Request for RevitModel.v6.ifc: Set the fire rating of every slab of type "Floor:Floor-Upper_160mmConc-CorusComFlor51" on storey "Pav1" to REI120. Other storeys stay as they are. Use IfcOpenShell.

First a look at what the model holds.

```python
import ifcopenshell
import ifcopenshell.util.element

model = ifcopenshell.open("RevitModel.v6.ifc")
print(model.schema)
storey = next(s for s in model.by_type("IfcBuildingStorey") if s.Name == "Pav1")
slabs = [e for e in ifcopenshell.util.element.get_decomposition(storey) if e.is_a("IfcSlab")]
seen = {}
for e in slabs:
    element_type = ifcopenshell.util.element.get_type(e)
    key = (element_type.Name if element_type != e and element_type else None, ifcopenshell.util.element.get_pset(e, "Pset_SlabCommon", "FireRating"))
    seen[key] = seen.get(key, 0) + 1
for (name, value), count in sorted(seen.items(), key=str):
    print(count, "x", name, "|", value)
```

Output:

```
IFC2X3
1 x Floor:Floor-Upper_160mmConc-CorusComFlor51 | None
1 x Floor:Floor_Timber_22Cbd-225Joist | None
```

```python
import ifcopenshell
import ifcopenshell.api.pset
import ifcopenshell.util.element

model = ifcopenshell.open("RevitModel.v6.ifc")

storey = next(s for s in model.by_type("IfcBuildingStorey") if s.Name == "Pav1")
slabs = [e for e in ifcopenshell.util.element.get_decomposition(storey) if e.is_a("IfcSlab")]

count = 0
for e in slabs:
    element_type = ifcopenshell.util.element.get_type(e)
    if element_type in (None, e) or element_type.Name != "Floor:Floor-Upper_160mmConc-CorusComFlor51":
        continue
    # add_pset returns the element's existing set when there is one.
    pset = ifcopenshell.api.pset.add_pset(model, product=e, name="Pset_SlabCommon")
    ifcopenshell.api.pset.edit_pset(model, pset=pset, properties={"FireRating": "REI120"})
    count += 1

print(count, "slabs updated")

model.write("RevitModel.v6-out.ifc")
```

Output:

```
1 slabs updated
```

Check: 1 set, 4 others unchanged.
